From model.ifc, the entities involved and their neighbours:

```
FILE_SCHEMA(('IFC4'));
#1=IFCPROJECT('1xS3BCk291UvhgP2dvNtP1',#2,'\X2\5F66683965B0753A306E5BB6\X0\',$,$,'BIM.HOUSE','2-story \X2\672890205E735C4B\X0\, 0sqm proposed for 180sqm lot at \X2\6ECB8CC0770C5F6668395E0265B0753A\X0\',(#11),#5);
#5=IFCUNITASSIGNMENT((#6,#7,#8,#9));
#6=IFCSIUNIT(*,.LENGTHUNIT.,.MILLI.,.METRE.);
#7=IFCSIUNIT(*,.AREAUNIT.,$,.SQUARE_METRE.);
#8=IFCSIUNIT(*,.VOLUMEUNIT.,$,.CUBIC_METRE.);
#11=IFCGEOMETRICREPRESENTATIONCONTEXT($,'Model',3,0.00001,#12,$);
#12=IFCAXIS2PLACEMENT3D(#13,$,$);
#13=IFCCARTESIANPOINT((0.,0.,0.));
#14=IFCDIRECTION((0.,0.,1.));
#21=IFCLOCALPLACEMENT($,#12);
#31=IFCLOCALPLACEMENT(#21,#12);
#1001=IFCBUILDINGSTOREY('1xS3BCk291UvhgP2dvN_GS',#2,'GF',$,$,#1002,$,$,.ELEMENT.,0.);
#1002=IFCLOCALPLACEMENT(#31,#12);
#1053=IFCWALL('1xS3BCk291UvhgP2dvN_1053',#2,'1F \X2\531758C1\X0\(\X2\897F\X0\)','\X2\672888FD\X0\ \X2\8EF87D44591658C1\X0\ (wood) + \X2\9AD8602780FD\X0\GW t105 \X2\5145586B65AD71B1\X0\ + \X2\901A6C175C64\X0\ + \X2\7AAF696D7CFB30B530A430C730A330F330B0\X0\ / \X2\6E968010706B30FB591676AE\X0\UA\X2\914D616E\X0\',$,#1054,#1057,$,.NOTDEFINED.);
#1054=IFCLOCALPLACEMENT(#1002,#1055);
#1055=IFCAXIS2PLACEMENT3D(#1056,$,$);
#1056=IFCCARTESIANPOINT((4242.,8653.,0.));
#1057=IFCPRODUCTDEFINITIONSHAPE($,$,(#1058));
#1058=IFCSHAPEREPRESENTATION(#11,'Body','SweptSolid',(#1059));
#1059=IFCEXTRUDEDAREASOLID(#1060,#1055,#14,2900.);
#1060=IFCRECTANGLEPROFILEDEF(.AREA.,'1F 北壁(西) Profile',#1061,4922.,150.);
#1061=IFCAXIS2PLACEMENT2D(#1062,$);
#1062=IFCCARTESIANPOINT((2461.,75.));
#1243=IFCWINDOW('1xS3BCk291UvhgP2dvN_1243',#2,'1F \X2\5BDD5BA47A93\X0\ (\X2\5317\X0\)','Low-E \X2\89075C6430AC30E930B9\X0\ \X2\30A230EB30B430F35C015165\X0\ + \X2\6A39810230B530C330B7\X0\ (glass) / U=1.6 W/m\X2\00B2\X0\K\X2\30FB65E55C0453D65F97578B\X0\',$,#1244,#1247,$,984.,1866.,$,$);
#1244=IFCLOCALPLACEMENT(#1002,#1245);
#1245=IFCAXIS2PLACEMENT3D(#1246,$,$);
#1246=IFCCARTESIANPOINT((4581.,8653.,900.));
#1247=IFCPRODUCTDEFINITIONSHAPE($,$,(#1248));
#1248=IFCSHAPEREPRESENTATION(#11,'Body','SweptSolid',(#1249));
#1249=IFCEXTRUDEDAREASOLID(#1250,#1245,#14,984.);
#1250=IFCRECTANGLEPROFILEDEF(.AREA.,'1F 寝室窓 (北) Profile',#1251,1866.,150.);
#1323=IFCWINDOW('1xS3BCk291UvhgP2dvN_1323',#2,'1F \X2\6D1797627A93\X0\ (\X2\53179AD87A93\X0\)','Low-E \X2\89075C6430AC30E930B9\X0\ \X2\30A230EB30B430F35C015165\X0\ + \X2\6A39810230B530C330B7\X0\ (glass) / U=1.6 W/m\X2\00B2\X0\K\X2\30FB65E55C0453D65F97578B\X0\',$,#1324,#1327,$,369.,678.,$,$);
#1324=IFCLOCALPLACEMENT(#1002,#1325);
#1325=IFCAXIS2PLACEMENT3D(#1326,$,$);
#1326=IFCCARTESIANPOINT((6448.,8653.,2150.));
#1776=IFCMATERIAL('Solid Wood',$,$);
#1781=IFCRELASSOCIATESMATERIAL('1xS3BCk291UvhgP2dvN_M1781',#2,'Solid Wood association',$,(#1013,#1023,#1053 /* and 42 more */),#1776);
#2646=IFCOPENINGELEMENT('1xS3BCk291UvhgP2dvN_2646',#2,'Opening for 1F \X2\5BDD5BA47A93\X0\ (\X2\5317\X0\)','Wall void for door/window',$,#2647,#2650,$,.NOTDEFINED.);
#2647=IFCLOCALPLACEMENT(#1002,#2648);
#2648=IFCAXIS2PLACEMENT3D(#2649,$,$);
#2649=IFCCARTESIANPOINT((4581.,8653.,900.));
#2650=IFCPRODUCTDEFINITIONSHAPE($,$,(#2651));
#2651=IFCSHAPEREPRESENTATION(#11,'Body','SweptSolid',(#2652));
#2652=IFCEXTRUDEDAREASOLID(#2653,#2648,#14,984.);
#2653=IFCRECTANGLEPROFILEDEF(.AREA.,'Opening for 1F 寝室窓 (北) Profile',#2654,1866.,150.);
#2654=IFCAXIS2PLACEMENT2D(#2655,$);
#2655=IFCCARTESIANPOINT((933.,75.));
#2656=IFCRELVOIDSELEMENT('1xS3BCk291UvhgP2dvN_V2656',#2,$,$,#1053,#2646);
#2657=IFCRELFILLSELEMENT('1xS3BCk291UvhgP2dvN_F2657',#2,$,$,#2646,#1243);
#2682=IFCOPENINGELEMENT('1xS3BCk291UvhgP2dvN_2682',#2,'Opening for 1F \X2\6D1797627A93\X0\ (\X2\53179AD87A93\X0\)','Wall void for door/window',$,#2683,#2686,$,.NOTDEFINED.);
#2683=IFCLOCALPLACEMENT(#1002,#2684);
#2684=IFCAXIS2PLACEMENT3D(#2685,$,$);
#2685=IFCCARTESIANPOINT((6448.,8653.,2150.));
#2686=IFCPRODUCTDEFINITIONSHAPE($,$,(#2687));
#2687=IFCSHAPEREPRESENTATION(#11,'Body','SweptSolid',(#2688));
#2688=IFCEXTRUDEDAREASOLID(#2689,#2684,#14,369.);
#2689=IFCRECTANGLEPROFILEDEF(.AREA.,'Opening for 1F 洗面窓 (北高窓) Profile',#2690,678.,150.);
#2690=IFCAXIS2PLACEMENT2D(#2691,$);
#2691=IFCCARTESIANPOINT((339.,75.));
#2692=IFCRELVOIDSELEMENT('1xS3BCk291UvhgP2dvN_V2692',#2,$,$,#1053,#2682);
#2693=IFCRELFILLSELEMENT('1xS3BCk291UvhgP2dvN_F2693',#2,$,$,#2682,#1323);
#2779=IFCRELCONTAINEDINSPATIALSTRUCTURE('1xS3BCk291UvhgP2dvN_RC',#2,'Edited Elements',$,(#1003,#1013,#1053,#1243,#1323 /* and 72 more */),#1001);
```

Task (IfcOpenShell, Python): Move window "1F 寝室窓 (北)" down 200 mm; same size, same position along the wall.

```python
import numpy as np
import ifcopenshell
import ifcopenshell.api.geometry
import ifcopenshell.util.placement
import ifcopenshell.util.unit

model = ifcopenshell.open("model.ifc")
unit_scale = ifcopenshell.util.unit.calculate_unit_scale(model)

window = model.by_guid("1xS3BCk291UvhgP2dvN_1243")
opening = window.FillsVoids[0].RelatingOpeningElement
dz = -200.0

shift = np.array([0.0, 0.0, dz])
# The window is not placed relative to its opening, so move both.
for product in (opening, window):
    matrix = ifcopenshell.util.placement.get_local_placement(product.ObjectPlacement)
    matrix[:3, 3] += shift
    ifcopenshell.api.geometry.edit_object_placement(model, product=product, matrix=matrix, is_si=False)

print(f"moved by {dz * unit_scale:+.3f} m")

model.write("model_rev.ifc")
```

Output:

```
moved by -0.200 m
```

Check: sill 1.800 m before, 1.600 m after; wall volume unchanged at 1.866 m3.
